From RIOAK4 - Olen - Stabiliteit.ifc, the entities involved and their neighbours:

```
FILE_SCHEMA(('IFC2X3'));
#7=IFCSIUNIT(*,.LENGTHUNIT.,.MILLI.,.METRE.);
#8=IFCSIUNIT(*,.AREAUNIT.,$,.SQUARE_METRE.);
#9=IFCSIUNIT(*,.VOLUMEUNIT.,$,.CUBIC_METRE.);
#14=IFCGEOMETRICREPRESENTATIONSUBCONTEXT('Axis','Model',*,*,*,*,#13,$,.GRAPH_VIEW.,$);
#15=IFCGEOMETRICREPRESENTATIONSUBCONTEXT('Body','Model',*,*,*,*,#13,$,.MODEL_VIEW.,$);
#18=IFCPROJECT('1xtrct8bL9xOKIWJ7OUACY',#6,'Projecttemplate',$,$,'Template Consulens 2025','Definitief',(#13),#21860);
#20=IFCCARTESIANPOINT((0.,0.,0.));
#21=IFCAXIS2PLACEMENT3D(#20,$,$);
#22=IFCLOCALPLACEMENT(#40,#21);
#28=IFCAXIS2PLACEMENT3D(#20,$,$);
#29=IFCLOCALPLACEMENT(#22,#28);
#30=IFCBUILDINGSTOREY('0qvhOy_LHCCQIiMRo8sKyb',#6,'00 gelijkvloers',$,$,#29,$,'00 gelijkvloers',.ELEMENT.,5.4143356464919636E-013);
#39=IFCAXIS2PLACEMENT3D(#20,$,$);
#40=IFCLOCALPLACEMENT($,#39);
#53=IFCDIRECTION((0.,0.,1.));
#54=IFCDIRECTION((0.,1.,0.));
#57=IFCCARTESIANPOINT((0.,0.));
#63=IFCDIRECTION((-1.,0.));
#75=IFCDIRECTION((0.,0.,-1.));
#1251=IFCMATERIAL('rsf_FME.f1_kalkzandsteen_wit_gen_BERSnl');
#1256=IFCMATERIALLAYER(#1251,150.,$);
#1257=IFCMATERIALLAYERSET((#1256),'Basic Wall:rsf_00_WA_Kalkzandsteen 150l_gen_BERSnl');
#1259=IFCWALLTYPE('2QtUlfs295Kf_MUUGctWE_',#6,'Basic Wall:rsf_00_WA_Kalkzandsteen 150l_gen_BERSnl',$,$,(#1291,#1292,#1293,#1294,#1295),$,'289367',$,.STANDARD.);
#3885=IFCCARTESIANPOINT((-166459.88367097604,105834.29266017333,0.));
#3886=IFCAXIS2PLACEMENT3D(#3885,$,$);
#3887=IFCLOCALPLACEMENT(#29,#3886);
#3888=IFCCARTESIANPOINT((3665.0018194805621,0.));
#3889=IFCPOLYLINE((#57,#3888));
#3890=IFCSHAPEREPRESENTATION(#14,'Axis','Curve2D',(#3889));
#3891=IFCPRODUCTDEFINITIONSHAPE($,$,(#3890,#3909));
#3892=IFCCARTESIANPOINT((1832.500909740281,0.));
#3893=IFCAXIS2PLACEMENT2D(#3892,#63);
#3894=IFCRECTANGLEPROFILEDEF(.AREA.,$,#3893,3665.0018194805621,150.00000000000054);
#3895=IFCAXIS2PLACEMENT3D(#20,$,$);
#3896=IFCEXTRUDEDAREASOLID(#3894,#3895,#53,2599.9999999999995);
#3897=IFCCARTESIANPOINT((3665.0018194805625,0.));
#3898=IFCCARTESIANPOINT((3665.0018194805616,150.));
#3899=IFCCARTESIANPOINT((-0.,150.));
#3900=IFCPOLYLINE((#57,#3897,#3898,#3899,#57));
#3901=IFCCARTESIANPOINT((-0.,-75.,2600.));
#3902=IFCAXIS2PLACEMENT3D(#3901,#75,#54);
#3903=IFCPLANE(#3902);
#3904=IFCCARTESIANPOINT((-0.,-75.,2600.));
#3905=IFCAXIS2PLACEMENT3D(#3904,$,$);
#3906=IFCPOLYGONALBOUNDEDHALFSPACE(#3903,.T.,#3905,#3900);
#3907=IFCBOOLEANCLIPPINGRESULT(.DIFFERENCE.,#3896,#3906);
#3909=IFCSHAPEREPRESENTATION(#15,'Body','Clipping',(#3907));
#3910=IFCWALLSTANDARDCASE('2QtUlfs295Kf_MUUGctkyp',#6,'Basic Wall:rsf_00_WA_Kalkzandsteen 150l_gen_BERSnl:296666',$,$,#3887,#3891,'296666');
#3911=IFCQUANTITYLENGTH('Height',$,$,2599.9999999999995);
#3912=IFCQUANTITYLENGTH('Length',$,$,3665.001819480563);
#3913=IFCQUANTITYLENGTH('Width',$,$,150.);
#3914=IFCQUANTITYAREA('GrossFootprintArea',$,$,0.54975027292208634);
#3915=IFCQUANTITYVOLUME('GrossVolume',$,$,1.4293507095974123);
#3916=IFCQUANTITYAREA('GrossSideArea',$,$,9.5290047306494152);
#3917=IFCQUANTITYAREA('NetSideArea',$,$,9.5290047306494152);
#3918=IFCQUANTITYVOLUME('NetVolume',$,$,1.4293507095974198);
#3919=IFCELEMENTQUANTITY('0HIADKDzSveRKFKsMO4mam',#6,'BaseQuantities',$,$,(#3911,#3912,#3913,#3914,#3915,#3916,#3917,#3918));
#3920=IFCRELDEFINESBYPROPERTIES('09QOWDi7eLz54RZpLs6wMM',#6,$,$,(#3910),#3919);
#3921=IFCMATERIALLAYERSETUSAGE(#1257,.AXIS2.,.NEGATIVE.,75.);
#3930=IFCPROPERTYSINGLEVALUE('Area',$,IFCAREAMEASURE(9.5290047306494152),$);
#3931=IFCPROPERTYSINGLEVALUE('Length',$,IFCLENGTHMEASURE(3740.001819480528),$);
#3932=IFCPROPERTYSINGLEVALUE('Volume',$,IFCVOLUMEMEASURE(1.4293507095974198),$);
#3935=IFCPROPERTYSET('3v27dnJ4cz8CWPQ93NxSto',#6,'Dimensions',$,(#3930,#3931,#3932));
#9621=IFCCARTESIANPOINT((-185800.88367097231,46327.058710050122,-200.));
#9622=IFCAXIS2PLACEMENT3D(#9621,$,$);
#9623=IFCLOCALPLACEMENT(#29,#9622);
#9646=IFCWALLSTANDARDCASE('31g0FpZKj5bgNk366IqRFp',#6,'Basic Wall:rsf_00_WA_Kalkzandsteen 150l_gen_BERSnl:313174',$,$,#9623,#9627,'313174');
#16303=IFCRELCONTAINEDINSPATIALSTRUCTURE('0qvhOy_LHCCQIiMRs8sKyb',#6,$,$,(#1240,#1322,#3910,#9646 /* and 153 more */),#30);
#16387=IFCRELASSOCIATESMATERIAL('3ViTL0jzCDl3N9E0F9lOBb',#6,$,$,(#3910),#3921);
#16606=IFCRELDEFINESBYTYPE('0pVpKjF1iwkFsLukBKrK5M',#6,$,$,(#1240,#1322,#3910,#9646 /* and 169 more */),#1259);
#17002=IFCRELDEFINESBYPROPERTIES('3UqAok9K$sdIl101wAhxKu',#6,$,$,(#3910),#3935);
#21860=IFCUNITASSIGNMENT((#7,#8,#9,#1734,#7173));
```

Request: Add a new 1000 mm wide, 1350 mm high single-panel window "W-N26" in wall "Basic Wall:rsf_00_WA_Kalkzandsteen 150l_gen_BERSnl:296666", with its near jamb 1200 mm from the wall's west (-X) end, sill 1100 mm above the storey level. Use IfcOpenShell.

```python
import numpy as np
import ifcopenshell
import ifcopenshell.api.feature
import ifcopenshell.api.geometry
import ifcopenshell.api.pset
import ifcopenshell.api.root
import ifcopenshell.api.spatial
import ifcopenshell.api.type
import ifcopenshell.geom
import ifcopenshell.util.element
import ifcopenshell.util.placement
import ifcopenshell.util.representation
import ifcopenshell.util.shape
import ifcopenshell.util.unit

model = ifcopenshell.open("RIOAK4 - Olen - Stabiliteit.ifc")
unit_scale = ifcopenshell.util.unit.calculate_unit_scale(model)
area_scale = ifcopenshell.util.unit.calculate_unit_scale(model, "AREAUNIT")
volume_scale = ifcopenshell.util.unit.calculate_unit_scale(model, "VOLUMEUNIT")
settings = ifcopenshell.geom.settings()


def volume(element):
    """Net volume in cubic metres, openings subtracted."""
    shape = ifcopenshell.geom.create_shape(settings, element)
    return ifcopenshell.util.shape.get_volume(shape.geometry)


wall = model.by_guid("2QtUlfs295Kf_MUUGctkyp")
storey = ifcopenshell.util.element.get_container(wall, ifc_class="IfcBuildingStorey")
context = ifcopenshell.util.representation.get_context(model, "Model", "Body", "MODEL_VIEW")
before = volume(wall)

width, height, from_end, sill = 1, 1.35, 1.2, 1.1  # metres

# The wall runs along its own X axis, and the end named is its -X end.
wall_shape = ifcopenshell.geom.create_shape(settings, wall)
x, y, z = ifcopenshell.util.shape.get_vertices(wall_shape.geometry).T
start = x.min() + from_end
face, thickness = float(y.min()), float(y.max() - y.min())
wall_matrix = ifcopenshell.util.placement.get_local_placement(wall.ObjectPlacement)
level = ifcopenshell.util.placement.get_local_placement(storey.ObjectPlacement)[2, 3]


def in_wall(x, y):
    """Placement at x, y metres in the wall's axes, at sill height."""
    matrix = wall_matrix.copy()
    matrix[:, 3] = wall_matrix @ np.array([x / unit_scale, y / unit_scale, 0.0, 1.0])
    matrix[2, 3] = level + sill / unit_scale
    return matrix


# Opening: a box that overshoots both wall faces by 50 mm.
opening = ifcopenshell.api.root.create_entity(model, ifc_class="IfcOpeningElement")
box = ifcopenshell.api.geometry.add_wall_representation(
    model, context=context, length=width, height=height, thickness=thickness + 0.1
)
ifcopenshell.api.geometry.assign_representation(model, product=opening, representation=box)
ifcopenshell.api.geometry.edit_object_placement(model, product=opening, matrix=in_wall(start, face - 0.05), is_si=False)
ifcopenshell.api.feature.add_feature(model, feature=opening, element=wall)

window = ifcopenshell.api.root.create_entity(model, ifc_class="IfcWindow", name="W-N26")
window.OverallWidth, window.OverallHeight = width / unit_scale, height / unit_scale
body = ifcopenshell.api.geometry.add_window_representation(
    model,
    context=context,
    overall_width=window.OverallWidth,
    overall_height=window.OverallHeight,
    partition_type="SINGLE_PANEL",
)
ifcopenshell.api.geometry.assign_representation(model, product=window, representation=body)
ifcopenshell.api.spatial.assign_container(model, products=[window], relating_structure=storey)
fills = ifcopenshell.api.feature.add_filling(model, opening=opening, element=window)
fills.OwnerHistory = window.OwnerHistory  # required in IFC2X3

# IFC2X3 keeps the operation on the window style.
style = ifcopenshell.api.root.create_entity(model, ifc_class="IfcWindowStyle", name="W-N26")
style.OperationType, style.ConstructionType = "SINGLE_PANEL", "NOTDEFINED"
style.ParameterTakesPrecedence = style.Sizeable = False
ifcopenshell.api.type.assign_type(model, related_objects=[window], relating_type=style)

# Centre the window in the wall's thickness.
ifcopenshell.api.geometry.edit_object_placement(model, product=window, matrix=in_wall(start, face), is_si=False)
window_shape = ifcopenshell.geom.create_shape(settings, window)
depth = ifcopenshell.util.shape.get_vertices(window_shape.geometry)[:, 1]
offset = face + thickness / 2 - (depth.min() + depth.max()) / 2
ifcopenshell.api.geometry.edit_object_placement(model, product=window, matrix=in_wall(start, offset), is_si=False)

after = volume(wall)

# Update the wall's stored quantities.
qto = model.by_id(ifcopenshell.util.element.get_pset(wall, "BaseQuantities", should_inherit=False)["id"])
ifcopenshell.api.pset.edit_qto(model, qto=qto, properties={
    "NetSideArea": after / thickness / area_scale,
    "NetVolume": after / volume_scale,
})
pset = model.by_id(ifcopenshell.util.element.get_pset(wall, "Dimensions", should_inherit=False)["id"])
ifcopenshell.api.pset.edit_pset(model, pset=pset, properties={
    "Area": model.create_entity("IfcAreaMeasure", after / thickness / area_scale),
    "Volume": model.create_entity("IfcVolumeMeasure", after / volume_scale),
})

print(f"wall volume {before:.3f} -> {after:.3f} m3")

model.write("RIOAK4 - Olen - Stabiliteit-out.ifc")
```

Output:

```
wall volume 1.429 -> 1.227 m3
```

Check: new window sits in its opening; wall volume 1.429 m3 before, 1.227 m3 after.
